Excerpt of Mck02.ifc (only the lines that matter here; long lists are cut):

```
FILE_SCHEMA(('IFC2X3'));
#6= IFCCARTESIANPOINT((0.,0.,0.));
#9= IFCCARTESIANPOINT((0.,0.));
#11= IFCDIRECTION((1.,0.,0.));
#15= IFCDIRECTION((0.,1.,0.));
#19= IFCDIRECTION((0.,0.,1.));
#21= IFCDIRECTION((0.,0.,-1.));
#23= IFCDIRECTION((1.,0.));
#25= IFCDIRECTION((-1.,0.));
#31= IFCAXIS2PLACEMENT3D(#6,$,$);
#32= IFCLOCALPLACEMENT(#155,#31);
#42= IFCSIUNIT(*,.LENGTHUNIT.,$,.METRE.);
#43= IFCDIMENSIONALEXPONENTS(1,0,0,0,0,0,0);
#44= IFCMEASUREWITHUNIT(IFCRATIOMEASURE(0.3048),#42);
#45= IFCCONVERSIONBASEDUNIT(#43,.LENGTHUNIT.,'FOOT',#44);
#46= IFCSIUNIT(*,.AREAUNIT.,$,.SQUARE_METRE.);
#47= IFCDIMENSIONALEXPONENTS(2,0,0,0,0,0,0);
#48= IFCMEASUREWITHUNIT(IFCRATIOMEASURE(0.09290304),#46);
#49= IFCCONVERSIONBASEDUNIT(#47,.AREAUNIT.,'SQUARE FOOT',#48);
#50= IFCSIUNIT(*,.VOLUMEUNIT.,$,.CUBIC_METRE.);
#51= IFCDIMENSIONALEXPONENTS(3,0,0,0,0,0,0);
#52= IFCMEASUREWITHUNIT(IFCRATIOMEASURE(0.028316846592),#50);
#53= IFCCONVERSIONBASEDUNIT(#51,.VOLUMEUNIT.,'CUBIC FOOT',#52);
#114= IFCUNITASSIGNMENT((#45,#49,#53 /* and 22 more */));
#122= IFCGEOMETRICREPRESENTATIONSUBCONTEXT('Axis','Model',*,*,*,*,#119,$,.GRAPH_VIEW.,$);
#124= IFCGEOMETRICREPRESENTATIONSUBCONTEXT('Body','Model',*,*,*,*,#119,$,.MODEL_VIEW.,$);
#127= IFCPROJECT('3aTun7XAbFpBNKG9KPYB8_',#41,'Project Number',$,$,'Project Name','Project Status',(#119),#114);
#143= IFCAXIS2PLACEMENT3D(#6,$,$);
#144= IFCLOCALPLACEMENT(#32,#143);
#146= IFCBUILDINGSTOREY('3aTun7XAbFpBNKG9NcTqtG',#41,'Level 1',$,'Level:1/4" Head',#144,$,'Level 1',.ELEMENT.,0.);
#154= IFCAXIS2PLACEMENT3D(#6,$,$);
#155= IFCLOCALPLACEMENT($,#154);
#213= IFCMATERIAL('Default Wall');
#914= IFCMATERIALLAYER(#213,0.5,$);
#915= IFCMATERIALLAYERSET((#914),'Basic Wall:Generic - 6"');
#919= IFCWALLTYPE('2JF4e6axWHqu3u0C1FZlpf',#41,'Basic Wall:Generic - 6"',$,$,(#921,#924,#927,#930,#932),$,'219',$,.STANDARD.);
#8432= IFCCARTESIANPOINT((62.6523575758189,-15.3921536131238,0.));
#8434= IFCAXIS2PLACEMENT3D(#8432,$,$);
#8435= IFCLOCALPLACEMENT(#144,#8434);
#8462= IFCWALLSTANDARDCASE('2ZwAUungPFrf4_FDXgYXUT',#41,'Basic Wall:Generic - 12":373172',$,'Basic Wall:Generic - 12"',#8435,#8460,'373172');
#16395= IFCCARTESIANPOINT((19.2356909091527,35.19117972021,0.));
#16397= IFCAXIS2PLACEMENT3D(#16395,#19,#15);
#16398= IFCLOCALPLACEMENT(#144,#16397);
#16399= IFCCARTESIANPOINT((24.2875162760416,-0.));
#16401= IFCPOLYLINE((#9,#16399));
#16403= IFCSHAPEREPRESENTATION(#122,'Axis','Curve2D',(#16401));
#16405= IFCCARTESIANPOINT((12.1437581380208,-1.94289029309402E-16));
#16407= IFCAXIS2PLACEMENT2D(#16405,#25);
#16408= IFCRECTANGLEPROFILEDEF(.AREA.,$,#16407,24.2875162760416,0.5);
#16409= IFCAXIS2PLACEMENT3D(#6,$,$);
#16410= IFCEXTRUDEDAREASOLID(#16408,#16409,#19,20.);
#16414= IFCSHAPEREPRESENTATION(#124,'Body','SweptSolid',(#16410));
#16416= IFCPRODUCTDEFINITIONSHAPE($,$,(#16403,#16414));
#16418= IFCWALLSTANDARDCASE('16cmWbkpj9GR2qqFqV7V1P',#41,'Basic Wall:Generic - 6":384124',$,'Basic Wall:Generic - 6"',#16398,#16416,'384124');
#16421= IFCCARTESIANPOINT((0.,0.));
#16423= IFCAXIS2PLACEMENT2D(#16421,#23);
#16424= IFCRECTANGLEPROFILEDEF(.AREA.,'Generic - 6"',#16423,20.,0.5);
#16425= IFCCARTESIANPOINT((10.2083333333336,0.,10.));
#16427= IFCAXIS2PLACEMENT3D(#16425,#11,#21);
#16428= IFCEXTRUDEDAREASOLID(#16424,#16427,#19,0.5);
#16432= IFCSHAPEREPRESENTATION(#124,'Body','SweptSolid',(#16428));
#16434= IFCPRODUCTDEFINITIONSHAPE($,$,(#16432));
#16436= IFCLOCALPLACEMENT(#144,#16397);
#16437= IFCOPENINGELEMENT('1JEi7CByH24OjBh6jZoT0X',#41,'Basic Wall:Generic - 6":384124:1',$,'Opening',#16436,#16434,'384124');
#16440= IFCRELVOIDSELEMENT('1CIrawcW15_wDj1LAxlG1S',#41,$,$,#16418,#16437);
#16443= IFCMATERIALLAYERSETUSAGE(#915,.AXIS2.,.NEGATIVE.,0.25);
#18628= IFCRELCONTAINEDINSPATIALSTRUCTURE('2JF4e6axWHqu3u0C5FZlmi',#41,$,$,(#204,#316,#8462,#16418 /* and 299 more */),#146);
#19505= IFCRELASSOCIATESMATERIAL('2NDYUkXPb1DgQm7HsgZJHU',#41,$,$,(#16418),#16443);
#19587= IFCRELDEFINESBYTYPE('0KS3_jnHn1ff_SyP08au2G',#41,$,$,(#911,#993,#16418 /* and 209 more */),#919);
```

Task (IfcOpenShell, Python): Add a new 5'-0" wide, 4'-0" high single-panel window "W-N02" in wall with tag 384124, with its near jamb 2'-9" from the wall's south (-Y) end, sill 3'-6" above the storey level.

```python
import numpy as np
import ifcopenshell
import ifcopenshell.api.feature
import ifcopenshell.api.geometry
import ifcopenshell.api.root
import ifcopenshell.api.spatial
import ifcopenshell.api.type
import ifcopenshell.geom
import ifcopenshell.util.element
import ifcopenshell.util.placement
import ifcopenshell.util.representation
import ifcopenshell.util.shape
import ifcopenshell.util.unit

model = ifcopenshell.open("Mck02.ifc")
unit_scale = ifcopenshell.util.unit.calculate_unit_scale(model)
settings = ifcopenshell.geom.settings()


def volume(element):
    """Net volume in cubic metres, openings subtracted."""
    shape = ifcopenshell.geom.create_shape(settings, element)
    return ifcopenshell.util.shape.get_volume(shape.geometry)


wall = model.by_guid("16cmWbkpj9GR2qqFqV7V1P")
storey = ifcopenshell.util.element.get_container(wall, ifc_class="IfcBuildingStorey")
context = ifcopenshell.util.representation.get_context(model, "Model", "Body", "MODEL_VIEW")
before = volume(wall)

width, height, from_end, sill = 1.524, 1.2192, 0.8382, 1.0668  # metres

# The wall runs along its own X axis, and the end named is its -X end.
wall_shape = ifcopenshell.geom.create_shape(settings, wall)
x, y, z = ifcopenshell.util.shape.get_vertices(wall_shape.geometry).T
start = x.min() + from_end
face, thickness = float(y.min()), float(y.max() - y.min())
wall_matrix = ifcopenshell.util.placement.get_local_placement(wall.ObjectPlacement)
level = ifcopenshell.util.placement.get_local_placement(storey.ObjectPlacement)[2, 3]


def in_wall(x, y):
    """Placement at x, y metres in the wall's axes, at sill height."""
    matrix = wall_matrix.copy()
    matrix[:, 3] = wall_matrix @ np.array([x / unit_scale, y / unit_scale, 0.0, 1.0])
    matrix[2, 3] = level + sill / unit_scale
    return matrix


# Opening: a box that overshoots both wall faces by 50 mm.
opening = ifcopenshell.api.root.create_entity(model, ifc_class="IfcOpeningElement")
box = ifcopenshell.api.geometry.add_wall_representation(
    model, context=context, length=width, height=height, thickness=thickness + 0.1
)
ifcopenshell.api.geometry.assign_representation(model, product=opening, representation=box)
ifcopenshell.api.geometry.edit_object_placement(model, product=opening, matrix=in_wall(start, face - 0.05), is_si=False)
ifcopenshell.api.feature.add_feature(model, feature=opening, element=wall)

window = ifcopenshell.api.root.create_entity(model, ifc_class="IfcWindow", name="W-N02")
window.OverallWidth, window.OverallHeight = width / unit_scale, height / unit_scale
body = ifcopenshell.api.geometry.add_window_representation(
    model,
    context=context,
    overall_width=window.OverallWidth,
    overall_height=window.OverallHeight,
    partition_type="SINGLE_PANEL",
)
ifcopenshell.api.geometry.assign_representation(model, product=window, representation=body)
ifcopenshell.api.spatial.assign_container(model, products=[window], relating_structure=storey)
fills = ifcopenshell.api.feature.add_filling(model, opening=opening, element=window)
fills.OwnerHistory = window.OwnerHistory  # required in IFC2X3

# IFC2X3 keeps the operation on the window style.
style = ifcopenshell.api.root.create_entity(model, ifc_class="IfcWindowStyle", name="W-N02")
style.OperationType, style.ConstructionType = "SINGLE_PANEL", "NOTDEFINED"
style.ParameterTakesPrecedence = style.Sizeable = False
ifcopenshell.api.type.assign_type(model, related_objects=[window], relating_type=style)

# Centre the window in the wall's thickness.
ifcopenshell.api.geometry.edit_object_placement(model, product=window, matrix=in_wall(start, face), is_si=False)
window_shape = ifcopenshell.geom.create_shape(settings, window)
depth = ifcopenshell.util.shape.get_vertices(window_shape.geometry)[:, 1]
offset = face + thickness / 2 - (depth.min() + depth.max()) / 2
ifcopenshell.api.geometry.edit_object_placement(model, product=window, matrix=in_wall(start, offset), is_si=False)

after = volume(wall)

print(f"wall volume {before:.3f} -> {after:.3f} m3")

model.write("Mck02_v2.ifc")
```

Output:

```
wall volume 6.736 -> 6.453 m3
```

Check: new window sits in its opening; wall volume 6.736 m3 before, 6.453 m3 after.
